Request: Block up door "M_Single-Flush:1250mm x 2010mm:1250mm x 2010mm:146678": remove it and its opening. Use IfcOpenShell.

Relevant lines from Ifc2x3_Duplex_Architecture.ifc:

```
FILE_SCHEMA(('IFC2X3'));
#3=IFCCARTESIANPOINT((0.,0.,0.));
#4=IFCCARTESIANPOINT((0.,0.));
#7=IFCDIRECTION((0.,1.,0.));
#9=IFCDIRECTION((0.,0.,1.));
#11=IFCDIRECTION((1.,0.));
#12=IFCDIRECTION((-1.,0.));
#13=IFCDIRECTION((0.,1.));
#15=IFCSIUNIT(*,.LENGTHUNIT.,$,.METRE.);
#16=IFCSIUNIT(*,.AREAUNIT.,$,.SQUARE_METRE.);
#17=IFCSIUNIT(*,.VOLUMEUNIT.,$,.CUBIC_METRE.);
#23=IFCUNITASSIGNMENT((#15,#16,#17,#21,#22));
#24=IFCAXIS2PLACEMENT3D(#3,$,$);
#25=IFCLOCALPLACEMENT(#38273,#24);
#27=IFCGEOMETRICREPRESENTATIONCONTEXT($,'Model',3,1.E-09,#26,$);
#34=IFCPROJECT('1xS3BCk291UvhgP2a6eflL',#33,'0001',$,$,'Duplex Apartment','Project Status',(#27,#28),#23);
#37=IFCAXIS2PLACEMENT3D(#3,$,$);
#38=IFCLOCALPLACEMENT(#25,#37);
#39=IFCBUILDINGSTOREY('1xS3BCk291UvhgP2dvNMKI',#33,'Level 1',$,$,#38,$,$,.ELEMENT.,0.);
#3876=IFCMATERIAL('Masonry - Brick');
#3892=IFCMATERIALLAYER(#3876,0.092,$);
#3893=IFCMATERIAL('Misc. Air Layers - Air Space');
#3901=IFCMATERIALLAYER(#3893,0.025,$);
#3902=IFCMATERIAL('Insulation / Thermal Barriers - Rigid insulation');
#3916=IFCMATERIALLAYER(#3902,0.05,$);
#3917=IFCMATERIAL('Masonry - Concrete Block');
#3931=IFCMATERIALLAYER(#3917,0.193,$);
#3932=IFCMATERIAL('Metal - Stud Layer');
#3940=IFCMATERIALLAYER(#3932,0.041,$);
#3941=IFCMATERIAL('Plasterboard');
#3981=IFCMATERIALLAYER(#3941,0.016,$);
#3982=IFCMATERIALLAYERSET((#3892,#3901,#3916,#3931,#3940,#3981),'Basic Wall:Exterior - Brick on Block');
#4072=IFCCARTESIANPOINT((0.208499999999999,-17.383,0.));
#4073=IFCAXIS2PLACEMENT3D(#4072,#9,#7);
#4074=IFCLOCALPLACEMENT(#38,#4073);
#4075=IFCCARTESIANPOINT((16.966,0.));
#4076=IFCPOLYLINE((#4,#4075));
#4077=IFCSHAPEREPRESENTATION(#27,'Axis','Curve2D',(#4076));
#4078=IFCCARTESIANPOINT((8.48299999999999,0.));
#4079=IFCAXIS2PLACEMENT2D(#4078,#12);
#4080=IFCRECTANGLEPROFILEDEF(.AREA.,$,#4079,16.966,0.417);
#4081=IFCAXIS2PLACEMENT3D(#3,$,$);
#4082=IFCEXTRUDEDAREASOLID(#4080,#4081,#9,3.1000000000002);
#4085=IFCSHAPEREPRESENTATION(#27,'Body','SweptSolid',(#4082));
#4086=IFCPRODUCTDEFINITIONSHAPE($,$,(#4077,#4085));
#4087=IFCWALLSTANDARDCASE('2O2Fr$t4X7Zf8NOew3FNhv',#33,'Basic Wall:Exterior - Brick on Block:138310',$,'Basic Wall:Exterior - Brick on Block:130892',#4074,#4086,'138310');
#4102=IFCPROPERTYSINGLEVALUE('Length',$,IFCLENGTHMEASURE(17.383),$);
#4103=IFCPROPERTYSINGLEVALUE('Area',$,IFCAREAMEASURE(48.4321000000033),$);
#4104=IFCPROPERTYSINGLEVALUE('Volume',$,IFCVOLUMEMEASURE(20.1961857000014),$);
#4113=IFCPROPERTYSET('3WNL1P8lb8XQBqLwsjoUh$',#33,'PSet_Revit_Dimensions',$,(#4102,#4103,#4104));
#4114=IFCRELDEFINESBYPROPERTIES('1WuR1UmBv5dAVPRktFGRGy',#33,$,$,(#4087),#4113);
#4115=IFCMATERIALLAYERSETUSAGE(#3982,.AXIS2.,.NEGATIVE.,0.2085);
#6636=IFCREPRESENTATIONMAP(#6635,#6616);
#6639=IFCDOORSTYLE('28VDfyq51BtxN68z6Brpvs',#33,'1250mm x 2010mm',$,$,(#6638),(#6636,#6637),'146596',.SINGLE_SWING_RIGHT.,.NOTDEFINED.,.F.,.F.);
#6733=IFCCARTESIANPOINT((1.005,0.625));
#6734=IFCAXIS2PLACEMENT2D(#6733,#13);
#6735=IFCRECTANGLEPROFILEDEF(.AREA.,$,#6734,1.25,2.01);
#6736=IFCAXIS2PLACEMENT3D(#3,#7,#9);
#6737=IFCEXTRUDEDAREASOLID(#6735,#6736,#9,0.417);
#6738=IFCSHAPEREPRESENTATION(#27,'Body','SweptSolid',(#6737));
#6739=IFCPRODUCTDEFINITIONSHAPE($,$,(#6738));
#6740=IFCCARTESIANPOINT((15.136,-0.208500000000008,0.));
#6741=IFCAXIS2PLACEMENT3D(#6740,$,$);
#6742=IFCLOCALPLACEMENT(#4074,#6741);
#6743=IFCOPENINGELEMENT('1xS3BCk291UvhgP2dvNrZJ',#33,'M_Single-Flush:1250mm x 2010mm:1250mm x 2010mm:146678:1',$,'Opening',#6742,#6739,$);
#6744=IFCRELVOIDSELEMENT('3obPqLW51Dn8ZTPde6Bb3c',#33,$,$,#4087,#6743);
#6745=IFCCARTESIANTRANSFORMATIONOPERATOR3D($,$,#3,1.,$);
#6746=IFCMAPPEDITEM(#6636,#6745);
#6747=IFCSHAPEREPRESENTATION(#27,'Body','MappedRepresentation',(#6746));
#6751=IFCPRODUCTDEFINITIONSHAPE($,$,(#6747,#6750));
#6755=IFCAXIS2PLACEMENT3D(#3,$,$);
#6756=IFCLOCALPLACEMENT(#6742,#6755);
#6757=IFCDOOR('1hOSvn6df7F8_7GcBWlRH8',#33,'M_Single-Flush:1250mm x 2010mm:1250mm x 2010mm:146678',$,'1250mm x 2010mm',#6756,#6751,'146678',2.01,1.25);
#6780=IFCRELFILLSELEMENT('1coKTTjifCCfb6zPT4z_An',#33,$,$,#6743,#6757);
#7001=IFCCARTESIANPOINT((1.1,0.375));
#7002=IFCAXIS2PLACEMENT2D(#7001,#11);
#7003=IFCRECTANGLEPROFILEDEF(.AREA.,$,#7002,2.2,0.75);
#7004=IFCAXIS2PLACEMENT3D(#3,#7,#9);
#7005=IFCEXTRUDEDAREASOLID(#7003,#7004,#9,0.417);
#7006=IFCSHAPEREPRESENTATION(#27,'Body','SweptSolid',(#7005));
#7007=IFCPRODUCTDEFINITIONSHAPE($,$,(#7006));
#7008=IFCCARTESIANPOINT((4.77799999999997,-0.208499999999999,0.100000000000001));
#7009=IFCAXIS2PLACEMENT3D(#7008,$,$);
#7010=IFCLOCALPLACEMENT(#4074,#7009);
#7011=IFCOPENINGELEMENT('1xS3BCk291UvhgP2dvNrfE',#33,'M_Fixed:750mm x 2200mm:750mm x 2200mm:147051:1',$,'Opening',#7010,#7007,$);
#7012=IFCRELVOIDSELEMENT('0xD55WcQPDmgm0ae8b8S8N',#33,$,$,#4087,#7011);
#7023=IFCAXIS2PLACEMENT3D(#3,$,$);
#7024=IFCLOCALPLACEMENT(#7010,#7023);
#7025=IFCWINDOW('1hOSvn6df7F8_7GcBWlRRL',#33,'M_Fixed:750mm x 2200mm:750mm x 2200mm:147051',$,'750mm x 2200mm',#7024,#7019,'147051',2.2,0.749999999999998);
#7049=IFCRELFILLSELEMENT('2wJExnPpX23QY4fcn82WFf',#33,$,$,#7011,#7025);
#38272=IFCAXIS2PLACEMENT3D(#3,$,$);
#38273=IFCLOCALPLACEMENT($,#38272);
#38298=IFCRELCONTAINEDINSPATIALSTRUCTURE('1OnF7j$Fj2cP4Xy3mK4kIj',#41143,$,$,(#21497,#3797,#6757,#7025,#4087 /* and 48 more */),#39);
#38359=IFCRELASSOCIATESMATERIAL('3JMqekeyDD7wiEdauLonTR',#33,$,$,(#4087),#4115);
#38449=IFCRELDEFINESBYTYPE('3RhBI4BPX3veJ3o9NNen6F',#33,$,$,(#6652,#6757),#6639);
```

```python
import ifcopenshell
import ifcopenshell.api.feature
import ifcopenshell.api.pset
import ifcopenshell.api.root
import ifcopenshell.geom
import ifcopenshell.util.element
import ifcopenshell.util.shape
import ifcopenshell.util.unit

model = ifcopenshell.open("Ifc2x3_Duplex_Architecture.ifc")
area_scale = ifcopenshell.util.unit.calculate_unit_scale(model, "AREAUNIT")
volume_scale = ifcopenshell.util.unit.calculate_unit_scale(model, "VOLUMEUNIT")
settings = ifcopenshell.geom.settings()


def volume(element):
    """Net volume in cubic metres, openings subtracted."""
    shape = ifcopenshell.geom.create_shape(settings, element)
    return ifcopenshell.util.shape.get_volume(shape.geometry)


door = model.by_id(6757)
opening = door.FillsVoids[0].RelatingOpeningElement
wall = opening.VoidsElements[0].RelatingBuildingElement
before = volume(wall)

ifcopenshell.api.root.remove_product(model, product=door)
ifcopenshell.api.feature.remove_feature(model, feature=opening)

after = volume(wall)
thickness = 0.417  # wall thickness in metres

# Update the wall's stored quantities.
pset = model.by_id(ifcopenshell.util.element.get_pset(wall, "PSet_Revit_Dimensions", should_inherit=False)["id"])
ifcopenshell.api.pset.edit_pset(model, pset=pset, properties={
    "Area": model.create_entity("IfcAreaMeasure", after / thickness / area_scale),
    "Volume": model.create_entity("IfcVolumeMeasure", after / volume_scale),
})

print(f"wall volume {before:.3f} -> {after:.3f} m3")

model.write("Ifc2x3_Duplex_Architecture_edited.ifc")
```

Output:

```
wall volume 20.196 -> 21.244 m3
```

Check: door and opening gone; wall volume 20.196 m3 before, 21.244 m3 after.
